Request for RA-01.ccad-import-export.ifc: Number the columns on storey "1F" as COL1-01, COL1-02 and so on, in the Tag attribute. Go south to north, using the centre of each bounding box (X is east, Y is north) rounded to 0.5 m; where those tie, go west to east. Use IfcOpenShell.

First a look at what the model holds.

```python
import ifcopenshell
import ifcopenshell.util.element
import ifcopenshell.util.placement

model = ifcopenshell.open("RA-01.ccad-import-export.ifc")
print(model.schema)
storey = next(s for s in model.by_type("IfcBuildingStorey") if s.Name == "1F")
columns = [e for e in ifcopenshell.util.element.get_decomposition(storey) if e.is_a("IfcColumn")]
for e in sorted(columns, key=lambda e: e.id()):
    origin = ifcopenshell.util.placement.get_local_placement(e.ObjectPlacement)[:3, 3]
    print(e.id(), e.Tag, e.Name, origin.round(2) + 0.0, sep=" | ")
```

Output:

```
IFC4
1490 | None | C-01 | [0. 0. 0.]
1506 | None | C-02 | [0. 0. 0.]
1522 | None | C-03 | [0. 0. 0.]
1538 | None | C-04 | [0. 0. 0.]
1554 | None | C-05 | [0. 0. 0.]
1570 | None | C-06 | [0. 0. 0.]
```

```python
import ifcopenshell
import ifcopenshell.geom
import ifcopenshell.util.element
import ifcopenshell.util.shape

model = ifcopenshell.open("RA-01.ccad-import-export.ifc")
settings = ifcopenshell.geom.settings()
settings.set("use-world-coords", True)


def centre(element):
    shape = ifcopenshell.geom.create_shape(settings, element)
    return ifcopenshell.util.shape.get_bbox_centroid(shape.geometry)


storey = next(s for s in model.by_type("IfcBuildingStorey") if s.Name == "1F")
columns = [e for e in ifcopenshell.util.element.get_decomposition(storey) if e.is_a("IfcColumn")]

# Insertion points can sit at a corner or the storey origin, so sort by the geometry (in metres).
centres = {e: centre(e) for e in columns}
columns.sort(key=lambda e: (round(centres[e][1] / 0.5), centres[e][0]))

for i, e in enumerate(columns, start=1):
    number = f"COL1-{i:02d}"
    e.Tag = number
    print(e.id(), number)

model.write("RA-01.ccad-import-export_edited.ifc")
```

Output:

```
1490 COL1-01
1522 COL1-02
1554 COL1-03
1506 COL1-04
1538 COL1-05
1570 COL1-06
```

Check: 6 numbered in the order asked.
